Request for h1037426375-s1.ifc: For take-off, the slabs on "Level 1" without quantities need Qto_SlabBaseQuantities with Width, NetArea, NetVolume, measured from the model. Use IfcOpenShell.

First a look at what the model holds.

```python
import ifcopenshell
import ifcopenshell.util.element
import ifcopenshell.util.unit

model = ifcopenshell.open("h1037426375-s1.ifc")
print(model.schema)
for unit_type in ("LENGTHUNIT", "AREAUNIT", "VOLUMEUNIT"):
    print(unit_type, ifcopenshell.util.unit.calculate_unit_scale(model, unit_type))
storey = next(s for s in model.by_type("IfcBuildingStorey") if s.Name == "Level 1")
slabs = [e for e in ifcopenshell.util.element.get_decomposition(storey) if e.is_a("IfcSlab")]
for e in sorted(slabs, key=lambda e: e.id()):
    print(e.id(), e.is_a(), e.Name, list(ifcopenshell.util.element.get_psets(e, qtos_only=True)), sep=" | ")
```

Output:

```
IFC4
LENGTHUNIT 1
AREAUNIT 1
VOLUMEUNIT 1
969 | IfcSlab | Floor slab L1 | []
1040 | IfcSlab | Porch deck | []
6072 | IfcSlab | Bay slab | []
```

```python
import ifcopenshell
import ifcopenshell.api.pset
import ifcopenshell.geom
import ifcopenshell.util.element
import ifcopenshell.util.shape
import ifcopenshell.util.unit

model = ifcopenshell.open("h1037426375-s1.ifc")
unit_scale = ifcopenshell.util.unit.calculate_unit_scale(model)
area_scale = ifcopenshell.util.unit.calculate_unit_scale(model, "AREAUNIT")
volume_scale = ifcopenshell.util.unit.calculate_unit_scale(model, "VOLUMEUNIT")
settings = ifcopenshell.geom.settings()

storey = next(s for s in model.by_type("IfcBuildingStorey") if s.Name == "Level 1")
slabs = [e for e in ifcopenshell.util.element.get_decomposition(storey) if e.is_a("IfcSlab")]

for e in sorted(slabs, key=lambda e: e.id()):
    if ifcopenshell.util.element.get_psets(e, qtos_only=True, should_inherit=False):
        continue
    # Geometry comes back in metres, in the element's own axes.
    shape = ifcopenshell.geom.create_shape(settings, e)
    values = {
        "Width": ifcopenshell.util.shape.get_z(shape.geometry) / unit_scale,
        "NetArea": ifcopenshell.util.shape.get_footprint_area(shape.geometry) / area_scale,
        "NetVolume": ifcopenshell.util.shape.get_volume(shape.geometry) / volume_scale,
    }
    qto = ifcopenshell.api.pset.add_qto(model, product=e, name="Qto_SlabBaseQuantities")
    ifcopenshell.api.pset.edit_qto(model, qto=qto, properties=values)
    print(e.id(), {k: round(v, 3) for k, v in values.items()})

model.write("h1037426375-s1_rev.ifc")
```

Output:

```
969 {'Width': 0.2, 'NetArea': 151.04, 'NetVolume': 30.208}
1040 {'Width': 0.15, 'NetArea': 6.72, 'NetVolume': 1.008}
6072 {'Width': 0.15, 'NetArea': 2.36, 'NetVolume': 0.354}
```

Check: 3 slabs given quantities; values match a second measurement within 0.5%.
